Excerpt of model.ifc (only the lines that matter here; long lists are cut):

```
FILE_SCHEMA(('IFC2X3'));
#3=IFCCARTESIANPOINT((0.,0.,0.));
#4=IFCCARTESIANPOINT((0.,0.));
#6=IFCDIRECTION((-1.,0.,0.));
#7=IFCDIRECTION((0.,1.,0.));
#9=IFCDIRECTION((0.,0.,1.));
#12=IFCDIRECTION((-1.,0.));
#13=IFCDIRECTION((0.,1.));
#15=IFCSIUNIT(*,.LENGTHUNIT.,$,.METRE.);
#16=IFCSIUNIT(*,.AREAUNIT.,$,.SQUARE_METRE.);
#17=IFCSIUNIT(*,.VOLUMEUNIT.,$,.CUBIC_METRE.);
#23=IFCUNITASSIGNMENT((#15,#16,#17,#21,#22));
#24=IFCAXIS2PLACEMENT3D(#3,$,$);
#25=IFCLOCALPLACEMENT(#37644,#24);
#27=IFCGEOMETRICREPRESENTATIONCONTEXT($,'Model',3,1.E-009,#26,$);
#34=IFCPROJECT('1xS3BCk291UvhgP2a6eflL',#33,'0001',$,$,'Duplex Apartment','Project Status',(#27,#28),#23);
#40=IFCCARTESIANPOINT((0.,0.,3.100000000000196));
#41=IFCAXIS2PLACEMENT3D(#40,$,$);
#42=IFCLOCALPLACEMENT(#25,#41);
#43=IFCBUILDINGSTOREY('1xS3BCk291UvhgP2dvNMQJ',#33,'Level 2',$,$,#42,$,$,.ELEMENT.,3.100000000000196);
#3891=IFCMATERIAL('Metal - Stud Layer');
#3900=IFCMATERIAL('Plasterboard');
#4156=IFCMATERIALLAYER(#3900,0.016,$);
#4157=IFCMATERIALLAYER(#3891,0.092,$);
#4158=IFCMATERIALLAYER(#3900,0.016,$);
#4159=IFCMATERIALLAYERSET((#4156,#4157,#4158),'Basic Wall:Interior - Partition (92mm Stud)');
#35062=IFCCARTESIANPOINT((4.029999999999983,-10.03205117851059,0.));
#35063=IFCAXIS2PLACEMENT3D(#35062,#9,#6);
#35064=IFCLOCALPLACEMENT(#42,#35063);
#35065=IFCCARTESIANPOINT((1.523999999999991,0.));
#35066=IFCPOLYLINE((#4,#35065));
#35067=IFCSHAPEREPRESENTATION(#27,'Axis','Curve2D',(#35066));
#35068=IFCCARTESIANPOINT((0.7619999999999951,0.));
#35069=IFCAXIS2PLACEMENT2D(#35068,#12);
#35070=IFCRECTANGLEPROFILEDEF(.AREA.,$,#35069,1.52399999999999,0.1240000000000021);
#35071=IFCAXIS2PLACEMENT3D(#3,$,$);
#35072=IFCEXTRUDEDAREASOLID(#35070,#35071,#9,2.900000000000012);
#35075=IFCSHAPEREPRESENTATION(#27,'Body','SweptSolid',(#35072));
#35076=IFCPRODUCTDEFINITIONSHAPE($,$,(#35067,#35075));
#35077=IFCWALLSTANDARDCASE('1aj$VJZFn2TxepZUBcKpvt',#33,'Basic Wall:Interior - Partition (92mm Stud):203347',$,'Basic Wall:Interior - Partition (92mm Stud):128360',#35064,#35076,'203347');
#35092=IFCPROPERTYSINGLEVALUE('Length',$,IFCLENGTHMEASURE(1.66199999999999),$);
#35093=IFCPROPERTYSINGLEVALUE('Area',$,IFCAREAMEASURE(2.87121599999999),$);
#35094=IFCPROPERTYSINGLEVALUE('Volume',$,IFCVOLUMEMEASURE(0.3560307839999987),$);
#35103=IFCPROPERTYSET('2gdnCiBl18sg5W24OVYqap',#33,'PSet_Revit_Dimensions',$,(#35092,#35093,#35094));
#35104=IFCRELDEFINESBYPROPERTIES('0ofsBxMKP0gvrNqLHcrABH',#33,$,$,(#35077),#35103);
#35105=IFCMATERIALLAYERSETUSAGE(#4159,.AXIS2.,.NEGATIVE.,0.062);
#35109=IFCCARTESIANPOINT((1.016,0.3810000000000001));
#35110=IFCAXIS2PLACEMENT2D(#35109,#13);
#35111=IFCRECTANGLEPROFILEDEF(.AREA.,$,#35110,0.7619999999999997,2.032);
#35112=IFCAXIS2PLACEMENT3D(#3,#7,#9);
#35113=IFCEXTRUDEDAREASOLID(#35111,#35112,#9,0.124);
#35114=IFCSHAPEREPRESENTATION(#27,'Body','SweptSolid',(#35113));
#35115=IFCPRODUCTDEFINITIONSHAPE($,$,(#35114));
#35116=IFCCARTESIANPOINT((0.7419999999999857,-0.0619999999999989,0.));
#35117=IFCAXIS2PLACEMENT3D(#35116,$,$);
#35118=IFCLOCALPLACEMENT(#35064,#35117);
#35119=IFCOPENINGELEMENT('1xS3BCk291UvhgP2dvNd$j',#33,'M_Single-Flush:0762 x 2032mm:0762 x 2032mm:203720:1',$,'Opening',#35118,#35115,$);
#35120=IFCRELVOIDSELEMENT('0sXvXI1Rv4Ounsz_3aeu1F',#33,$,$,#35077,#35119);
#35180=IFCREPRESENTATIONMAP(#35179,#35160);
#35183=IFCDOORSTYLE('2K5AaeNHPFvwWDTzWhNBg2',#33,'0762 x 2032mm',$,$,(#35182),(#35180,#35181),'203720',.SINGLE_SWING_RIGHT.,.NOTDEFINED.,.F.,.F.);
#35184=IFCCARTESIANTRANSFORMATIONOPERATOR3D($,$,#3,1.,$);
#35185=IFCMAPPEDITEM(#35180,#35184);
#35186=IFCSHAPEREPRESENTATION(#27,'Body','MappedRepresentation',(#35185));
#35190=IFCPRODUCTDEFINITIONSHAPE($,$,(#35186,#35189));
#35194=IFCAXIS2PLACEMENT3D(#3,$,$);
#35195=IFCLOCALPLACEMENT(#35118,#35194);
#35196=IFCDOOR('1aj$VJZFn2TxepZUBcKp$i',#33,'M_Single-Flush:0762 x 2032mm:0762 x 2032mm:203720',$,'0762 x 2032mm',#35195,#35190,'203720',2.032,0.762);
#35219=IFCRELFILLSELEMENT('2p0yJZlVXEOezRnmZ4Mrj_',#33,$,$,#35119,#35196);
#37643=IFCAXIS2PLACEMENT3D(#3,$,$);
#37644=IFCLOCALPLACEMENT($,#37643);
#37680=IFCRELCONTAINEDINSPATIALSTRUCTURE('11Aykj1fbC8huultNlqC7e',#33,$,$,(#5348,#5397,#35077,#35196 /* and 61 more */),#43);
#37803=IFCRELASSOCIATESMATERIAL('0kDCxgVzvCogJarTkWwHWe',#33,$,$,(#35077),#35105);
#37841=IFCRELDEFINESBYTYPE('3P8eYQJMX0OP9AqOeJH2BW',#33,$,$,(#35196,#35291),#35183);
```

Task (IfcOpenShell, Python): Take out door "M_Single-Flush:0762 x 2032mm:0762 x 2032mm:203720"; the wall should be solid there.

```python
import ifcopenshell
import ifcopenshell.api.feature
import ifcopenshell.api.pset
import ifcopenshell.api.root
import ifcopenshell.geom
import ifcopenshell.util.element
import ifcopenshell.util.shape
import ifcopenshell.util.unit

model = ifcopenshell.open("model.ifc")
area_scale = ifcopenshell.util.unit.calculate_unit_scale(model, "AREAUNIT")
volume_scale = ifcopenshell.util.unit.calculate_unit_scale(model, "VOLUMEUNIT")
settings = ifcopenshell.geom.settings()


def volume(element):
    """Net volume in cubic metres, openings subtracted."""
    shape = ifcopenshell.geom.create_shape(settings, element)
    return ifcopenshell.util.shape.get_volume(shape.geometry)


door = model.by_guid("1aj$VJZFn2TxepZUBcKp$i")
opening = door.FillsVoids[0].RelatingOpeningElement
wall = opening.VoidsElements[0].RelatingBuildingElement
before = volume(wall)

ifcopenshell.api.root.remove_product(model, product=door)
ifcopenshell.api.feature.remove_feature(model, feature=opening)

after = volume(wall)
thickness = 0.124  # wall thickness in metres

# Update the wall's stored quantities.
pset = model.by_id(ifcopenshell.util.element.get_pset(wall, "PSet_Revit_Dimensions", should_inherit=False)["id"])
ifcopenshell.api.pset.edit_pset(model, pset=pset, properties={
    "Area": model.create_entity("IfcAreaMeasure", after / thickness / area_scale),
    "Volume": model.create_entity("IfcVolumeMeasure", after / volume_scale),
})

print(f"wall volume {before:.3f} -> {after:.3f} m3")

model.write("model_updated.ifc")
```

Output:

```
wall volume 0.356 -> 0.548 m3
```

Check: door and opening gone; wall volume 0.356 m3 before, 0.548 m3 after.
